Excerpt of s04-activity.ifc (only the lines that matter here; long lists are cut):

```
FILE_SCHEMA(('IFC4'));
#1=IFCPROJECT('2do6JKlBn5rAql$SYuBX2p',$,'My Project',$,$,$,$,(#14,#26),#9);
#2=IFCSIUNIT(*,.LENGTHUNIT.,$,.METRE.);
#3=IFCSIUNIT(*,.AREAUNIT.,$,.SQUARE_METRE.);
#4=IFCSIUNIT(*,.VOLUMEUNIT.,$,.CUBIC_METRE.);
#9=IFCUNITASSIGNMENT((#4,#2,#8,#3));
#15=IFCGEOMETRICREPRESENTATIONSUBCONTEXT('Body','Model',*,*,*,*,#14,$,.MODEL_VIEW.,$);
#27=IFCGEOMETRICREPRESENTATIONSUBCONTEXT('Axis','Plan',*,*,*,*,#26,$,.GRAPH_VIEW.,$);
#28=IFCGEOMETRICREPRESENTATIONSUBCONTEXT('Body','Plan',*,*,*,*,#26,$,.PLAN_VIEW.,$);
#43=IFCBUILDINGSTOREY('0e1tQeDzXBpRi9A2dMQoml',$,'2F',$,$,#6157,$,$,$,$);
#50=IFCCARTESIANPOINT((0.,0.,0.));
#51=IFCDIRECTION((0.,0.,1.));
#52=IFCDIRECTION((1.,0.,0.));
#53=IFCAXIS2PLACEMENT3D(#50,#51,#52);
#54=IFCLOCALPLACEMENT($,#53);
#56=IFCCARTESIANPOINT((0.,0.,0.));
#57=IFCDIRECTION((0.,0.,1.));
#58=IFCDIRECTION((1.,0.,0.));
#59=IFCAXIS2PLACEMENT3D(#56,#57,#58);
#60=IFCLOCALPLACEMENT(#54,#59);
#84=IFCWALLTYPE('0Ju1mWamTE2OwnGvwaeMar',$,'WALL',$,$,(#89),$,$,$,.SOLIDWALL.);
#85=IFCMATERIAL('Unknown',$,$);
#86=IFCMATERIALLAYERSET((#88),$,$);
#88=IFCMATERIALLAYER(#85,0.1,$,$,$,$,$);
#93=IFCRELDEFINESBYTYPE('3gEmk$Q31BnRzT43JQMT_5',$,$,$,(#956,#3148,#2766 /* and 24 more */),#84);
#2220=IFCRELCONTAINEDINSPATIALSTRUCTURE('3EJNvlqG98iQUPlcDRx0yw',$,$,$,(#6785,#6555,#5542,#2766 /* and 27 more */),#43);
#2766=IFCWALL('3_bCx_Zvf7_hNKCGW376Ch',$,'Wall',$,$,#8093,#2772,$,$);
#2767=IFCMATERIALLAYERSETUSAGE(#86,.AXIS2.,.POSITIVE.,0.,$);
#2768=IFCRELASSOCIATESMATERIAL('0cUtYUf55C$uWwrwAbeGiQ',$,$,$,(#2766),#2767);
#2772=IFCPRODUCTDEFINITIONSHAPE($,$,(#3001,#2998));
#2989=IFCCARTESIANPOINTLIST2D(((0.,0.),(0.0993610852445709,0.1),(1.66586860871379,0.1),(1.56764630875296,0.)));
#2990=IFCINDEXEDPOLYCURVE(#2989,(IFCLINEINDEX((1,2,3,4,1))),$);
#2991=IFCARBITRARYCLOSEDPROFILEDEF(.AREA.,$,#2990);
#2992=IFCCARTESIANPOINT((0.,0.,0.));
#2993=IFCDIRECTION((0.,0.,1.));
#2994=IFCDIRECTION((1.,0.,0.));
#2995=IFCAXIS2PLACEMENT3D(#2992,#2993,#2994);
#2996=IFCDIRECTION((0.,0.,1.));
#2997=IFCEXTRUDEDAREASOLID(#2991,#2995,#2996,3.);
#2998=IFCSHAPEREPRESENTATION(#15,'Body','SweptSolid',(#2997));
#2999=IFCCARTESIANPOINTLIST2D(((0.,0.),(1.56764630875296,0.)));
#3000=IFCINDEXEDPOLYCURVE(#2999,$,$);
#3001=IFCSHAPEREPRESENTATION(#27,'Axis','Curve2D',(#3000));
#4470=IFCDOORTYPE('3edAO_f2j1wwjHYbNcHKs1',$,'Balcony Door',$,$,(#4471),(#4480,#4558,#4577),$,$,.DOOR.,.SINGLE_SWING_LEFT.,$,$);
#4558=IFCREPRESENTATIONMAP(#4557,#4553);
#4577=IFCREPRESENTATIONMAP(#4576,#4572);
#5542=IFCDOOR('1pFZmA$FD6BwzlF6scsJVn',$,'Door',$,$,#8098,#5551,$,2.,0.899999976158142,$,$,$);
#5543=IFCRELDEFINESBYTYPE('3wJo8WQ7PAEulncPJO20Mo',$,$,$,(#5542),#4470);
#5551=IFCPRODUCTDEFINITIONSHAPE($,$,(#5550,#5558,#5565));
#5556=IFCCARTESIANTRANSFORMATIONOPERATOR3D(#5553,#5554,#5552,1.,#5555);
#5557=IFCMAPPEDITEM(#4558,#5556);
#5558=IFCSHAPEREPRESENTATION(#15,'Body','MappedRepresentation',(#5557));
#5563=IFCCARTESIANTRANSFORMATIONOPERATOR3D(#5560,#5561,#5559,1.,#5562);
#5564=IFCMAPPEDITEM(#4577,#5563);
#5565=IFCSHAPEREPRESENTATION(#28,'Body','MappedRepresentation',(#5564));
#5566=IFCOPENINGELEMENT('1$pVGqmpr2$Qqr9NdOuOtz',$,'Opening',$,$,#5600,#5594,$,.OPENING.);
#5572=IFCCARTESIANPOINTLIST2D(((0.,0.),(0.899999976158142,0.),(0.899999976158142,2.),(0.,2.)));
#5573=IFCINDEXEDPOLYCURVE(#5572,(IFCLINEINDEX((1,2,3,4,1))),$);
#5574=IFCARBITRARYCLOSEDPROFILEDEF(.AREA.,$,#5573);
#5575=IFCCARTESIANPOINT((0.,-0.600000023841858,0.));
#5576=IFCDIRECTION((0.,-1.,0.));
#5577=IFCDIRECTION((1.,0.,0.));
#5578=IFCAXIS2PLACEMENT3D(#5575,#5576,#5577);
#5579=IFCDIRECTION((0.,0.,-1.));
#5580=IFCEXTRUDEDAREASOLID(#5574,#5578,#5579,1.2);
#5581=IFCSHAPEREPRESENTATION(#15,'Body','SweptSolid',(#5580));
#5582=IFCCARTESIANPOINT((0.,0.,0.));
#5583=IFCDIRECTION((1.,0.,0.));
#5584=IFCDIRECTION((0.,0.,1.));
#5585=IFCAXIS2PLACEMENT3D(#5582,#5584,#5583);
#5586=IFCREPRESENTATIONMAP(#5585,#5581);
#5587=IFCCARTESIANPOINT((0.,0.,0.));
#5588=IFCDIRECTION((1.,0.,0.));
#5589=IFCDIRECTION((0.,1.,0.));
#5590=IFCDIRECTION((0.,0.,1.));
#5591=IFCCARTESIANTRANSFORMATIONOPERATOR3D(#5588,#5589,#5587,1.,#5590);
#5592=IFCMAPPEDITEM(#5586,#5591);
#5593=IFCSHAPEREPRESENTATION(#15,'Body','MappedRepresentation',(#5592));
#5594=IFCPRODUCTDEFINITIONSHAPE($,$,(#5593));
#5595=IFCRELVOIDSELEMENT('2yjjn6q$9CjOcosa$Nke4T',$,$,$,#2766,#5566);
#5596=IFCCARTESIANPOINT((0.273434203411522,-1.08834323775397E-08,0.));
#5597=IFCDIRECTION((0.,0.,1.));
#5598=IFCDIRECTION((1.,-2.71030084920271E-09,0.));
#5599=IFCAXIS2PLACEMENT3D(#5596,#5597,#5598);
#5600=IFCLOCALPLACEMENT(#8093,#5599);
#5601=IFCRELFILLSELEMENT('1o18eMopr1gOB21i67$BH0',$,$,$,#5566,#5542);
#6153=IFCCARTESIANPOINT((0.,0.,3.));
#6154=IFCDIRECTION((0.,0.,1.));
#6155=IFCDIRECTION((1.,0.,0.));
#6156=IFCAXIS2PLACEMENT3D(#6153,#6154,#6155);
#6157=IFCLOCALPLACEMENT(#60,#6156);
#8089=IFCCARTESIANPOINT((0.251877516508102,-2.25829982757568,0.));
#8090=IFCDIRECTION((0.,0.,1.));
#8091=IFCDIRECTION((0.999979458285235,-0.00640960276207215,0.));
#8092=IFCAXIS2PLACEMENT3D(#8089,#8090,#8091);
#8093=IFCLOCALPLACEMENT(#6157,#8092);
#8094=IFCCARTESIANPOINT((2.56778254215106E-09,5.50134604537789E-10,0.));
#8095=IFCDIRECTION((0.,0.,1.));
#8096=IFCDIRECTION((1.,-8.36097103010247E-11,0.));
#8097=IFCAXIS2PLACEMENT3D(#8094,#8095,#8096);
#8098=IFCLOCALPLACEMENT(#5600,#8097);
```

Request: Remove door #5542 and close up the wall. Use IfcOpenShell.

```python
import ifcopenshell
import ifcopenshell.api.feature
import ifcopenshell.api.root
import ifcopenshell.geom
import ifcopenshell.util.shape

model = ifcopenshell.open("s04-activity.ifc")
settings = ifcopenshell.geom.settings()


def volume(element):
    """Net volume in cubic metres, openings subtracted."""
    shape = ifcopenshell.geom.create_shape(settings, element)
    return ifcopenshell.util.shape.get_volume(shape.geometry)


door = model.by_guid("1pFZmA$FD6BwzlF6scsJVn")
opening = door.FillsVoids[0].RelatingOpeningElement
wall = opening.VoidsElements[0].RelatingBuildingElement
before = volume(wall)

ifcopenshell.api.root.remove_product(model, product=door)
ifcopenshell.api.feature.remove_feature(model, feature=opening)

after = volume(wall)

print(f"wall volume {before:.3f} -> {after:.3f} m3")

model.write("s04-activity_rev.ifc")
```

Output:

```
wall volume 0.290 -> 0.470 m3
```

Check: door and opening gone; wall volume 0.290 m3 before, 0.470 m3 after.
